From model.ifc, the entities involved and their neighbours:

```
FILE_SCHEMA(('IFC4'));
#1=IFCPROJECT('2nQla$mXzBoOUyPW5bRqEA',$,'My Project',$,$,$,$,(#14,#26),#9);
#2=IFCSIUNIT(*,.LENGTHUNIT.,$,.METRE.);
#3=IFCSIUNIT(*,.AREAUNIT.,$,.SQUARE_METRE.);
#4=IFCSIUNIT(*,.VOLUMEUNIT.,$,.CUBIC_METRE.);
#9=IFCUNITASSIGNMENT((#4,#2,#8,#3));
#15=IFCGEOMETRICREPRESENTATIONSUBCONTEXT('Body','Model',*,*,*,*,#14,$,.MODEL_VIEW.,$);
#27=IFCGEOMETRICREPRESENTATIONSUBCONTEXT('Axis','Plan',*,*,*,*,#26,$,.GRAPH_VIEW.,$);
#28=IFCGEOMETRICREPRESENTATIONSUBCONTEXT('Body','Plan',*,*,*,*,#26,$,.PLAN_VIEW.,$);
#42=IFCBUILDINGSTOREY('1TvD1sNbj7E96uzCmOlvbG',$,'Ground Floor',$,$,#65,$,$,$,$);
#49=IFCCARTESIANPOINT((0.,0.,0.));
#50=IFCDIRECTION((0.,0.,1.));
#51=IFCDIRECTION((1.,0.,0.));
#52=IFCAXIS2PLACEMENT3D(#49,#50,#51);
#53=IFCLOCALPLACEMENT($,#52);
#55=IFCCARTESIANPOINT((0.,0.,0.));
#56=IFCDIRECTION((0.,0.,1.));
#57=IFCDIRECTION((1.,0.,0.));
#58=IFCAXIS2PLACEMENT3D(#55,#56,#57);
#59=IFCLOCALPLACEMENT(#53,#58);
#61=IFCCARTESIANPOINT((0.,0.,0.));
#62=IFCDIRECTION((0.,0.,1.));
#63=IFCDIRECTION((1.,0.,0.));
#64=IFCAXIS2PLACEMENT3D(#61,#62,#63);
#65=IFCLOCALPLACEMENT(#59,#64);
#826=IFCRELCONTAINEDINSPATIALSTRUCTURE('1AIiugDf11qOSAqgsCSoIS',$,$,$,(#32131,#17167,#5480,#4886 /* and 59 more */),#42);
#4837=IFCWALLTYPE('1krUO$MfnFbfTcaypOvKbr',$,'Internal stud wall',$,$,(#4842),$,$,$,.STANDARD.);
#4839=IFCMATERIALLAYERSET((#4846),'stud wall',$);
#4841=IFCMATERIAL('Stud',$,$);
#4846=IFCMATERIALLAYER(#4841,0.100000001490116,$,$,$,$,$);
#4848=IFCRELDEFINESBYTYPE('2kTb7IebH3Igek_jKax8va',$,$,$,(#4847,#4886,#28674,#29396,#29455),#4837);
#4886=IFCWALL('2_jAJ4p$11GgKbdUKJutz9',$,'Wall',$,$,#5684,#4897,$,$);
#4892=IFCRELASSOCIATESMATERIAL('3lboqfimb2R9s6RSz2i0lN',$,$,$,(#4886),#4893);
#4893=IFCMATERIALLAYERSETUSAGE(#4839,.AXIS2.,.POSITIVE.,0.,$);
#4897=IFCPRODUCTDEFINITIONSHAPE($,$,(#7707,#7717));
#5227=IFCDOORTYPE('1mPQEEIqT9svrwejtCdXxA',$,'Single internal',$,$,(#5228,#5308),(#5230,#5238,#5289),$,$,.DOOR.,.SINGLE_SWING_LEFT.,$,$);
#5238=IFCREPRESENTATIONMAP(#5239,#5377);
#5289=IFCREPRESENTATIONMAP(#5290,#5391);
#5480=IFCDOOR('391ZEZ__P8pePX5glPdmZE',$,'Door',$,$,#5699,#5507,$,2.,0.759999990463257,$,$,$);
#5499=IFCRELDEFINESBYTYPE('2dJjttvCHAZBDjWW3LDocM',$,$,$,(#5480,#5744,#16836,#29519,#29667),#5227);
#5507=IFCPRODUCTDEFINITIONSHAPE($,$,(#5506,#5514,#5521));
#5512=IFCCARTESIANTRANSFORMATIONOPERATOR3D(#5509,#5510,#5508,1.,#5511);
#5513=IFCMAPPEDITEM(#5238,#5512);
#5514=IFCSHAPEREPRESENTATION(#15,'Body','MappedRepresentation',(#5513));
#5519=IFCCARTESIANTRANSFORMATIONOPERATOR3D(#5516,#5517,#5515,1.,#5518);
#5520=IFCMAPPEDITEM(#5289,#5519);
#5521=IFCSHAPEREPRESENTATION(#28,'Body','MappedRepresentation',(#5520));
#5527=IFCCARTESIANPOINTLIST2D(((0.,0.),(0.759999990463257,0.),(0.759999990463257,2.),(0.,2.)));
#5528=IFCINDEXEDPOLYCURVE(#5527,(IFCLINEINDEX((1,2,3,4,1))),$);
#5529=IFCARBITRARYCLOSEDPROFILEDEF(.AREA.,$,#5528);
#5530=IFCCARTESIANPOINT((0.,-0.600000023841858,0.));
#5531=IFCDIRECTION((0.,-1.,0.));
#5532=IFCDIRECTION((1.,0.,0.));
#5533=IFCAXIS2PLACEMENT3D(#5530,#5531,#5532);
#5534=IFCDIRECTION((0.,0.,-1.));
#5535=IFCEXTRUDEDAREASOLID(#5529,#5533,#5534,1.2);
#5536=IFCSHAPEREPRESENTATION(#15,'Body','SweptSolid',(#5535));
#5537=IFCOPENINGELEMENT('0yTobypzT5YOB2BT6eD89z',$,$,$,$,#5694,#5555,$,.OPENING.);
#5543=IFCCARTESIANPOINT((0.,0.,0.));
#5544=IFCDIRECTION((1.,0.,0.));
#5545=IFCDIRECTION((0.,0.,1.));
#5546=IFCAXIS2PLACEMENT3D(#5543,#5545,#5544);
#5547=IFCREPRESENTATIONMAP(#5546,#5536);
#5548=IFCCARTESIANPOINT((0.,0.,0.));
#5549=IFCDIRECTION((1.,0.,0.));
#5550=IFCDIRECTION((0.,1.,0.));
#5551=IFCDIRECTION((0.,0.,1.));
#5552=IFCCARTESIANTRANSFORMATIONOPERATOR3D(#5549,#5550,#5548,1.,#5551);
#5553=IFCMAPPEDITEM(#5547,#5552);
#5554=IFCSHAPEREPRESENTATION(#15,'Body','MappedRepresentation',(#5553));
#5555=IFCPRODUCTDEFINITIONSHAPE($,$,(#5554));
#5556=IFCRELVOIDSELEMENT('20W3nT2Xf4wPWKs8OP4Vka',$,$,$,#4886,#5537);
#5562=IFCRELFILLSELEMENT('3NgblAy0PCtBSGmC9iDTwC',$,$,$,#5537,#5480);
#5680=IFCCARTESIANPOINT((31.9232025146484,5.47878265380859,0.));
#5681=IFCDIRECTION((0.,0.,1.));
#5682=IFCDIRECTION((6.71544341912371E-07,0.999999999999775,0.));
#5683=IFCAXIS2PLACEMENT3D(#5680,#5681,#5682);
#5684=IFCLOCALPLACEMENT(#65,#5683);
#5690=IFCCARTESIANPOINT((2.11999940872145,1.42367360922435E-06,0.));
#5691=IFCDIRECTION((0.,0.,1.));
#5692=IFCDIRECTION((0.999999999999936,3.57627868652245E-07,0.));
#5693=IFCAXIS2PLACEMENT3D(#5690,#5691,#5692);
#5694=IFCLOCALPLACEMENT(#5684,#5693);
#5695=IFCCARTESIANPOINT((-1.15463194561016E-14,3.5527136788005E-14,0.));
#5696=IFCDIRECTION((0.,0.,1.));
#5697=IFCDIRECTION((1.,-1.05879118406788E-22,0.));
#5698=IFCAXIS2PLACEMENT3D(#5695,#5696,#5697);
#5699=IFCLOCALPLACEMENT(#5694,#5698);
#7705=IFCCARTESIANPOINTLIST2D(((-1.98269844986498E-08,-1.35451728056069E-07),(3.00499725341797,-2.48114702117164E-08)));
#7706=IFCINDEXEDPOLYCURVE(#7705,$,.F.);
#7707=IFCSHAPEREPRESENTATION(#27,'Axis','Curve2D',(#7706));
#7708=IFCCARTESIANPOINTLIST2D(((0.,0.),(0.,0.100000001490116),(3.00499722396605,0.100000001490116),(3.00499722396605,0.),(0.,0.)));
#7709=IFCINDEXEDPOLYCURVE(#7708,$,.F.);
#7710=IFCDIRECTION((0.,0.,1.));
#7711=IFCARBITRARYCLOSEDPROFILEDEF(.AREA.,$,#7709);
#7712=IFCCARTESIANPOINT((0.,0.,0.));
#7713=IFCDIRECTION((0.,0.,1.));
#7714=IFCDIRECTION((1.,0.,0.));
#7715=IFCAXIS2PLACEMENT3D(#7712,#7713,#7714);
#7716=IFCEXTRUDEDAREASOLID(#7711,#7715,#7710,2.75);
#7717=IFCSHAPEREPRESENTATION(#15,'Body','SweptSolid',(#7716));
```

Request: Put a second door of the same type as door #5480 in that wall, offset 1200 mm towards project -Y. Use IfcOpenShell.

```python
import ifcopenshell
import ifcopenshell.api.feature
import ifcopenshell.api.geometry
import ifcopenshell.api.root
import ifcopenshell.geom
import ifcopenshell.util.element
import ifcopenshell.util.placement
import ifcopenshell.util.shape
import ifcopenshell.util.unit

model = ifcopenshell.open("model.ifc")
unit_scale = ifcopenshell.util.unit.calculate_unit_scale(model)
settings = ifcopenshell.geom.settings()


def volume(element):
    """Net volume in cubic metres, openings subtracted."""
    shape = ifcopenshell.geom.create_shape(settings, element)
    return ifcopenshell.util.shape.get_volume(shape.geometry)


door = model.by_guid("391ZEZ__P8pePX5glPdmZE")
opening = door.FillsVoids[0].RelatingOpeningElement
wall = opening.VoidsElements[0].RelatingBuildingElement
before = volume(wall)
shift = ifcopenshell.util.placement.get_local_placement(wall.ObjectPlacement)[:3, 0] * -1.2 / unit_scale

# copy_class copies the void relationship, type, container and properties, but no geometry.
new_opening = ifcopenshell.api.root.copy_class(model, product=opening)
new_opening.Representation = ifcopenshell.util.element.copy_deep(
    model, opening.Representation, exclude=["IfcGeometricRepresentationContext", "IfcRepresentationMap"]
)
new_door = ifcopenshell.api.root.copy_class(model, product=door)
new_door.Representation = ifcopenshell.util.element.copy_deep(
    model, door.Representation, exclude=["IfcGeometricRepresentationContext", "IfcRepresentationMap"]
)
ifcopenshell.api.feature.add_filling(model, opening=new_opening, element=new_door)

for old, new in ((opening, new_opening), (door, new_door)):
    matrix = ifcopenshell.util.placement.get_local_placement(old.ObjectPlacement)
    matrix[:3, 3] += shift
    ifcopenshell.api.geometry.edit_object_placement(model, product=new, matrix=matrix, is_si=False)

after = volume(wall)

print(f"wall volume {before:.3f} -> {after:.3f} m3")

model.write("model_updated.ifc")
```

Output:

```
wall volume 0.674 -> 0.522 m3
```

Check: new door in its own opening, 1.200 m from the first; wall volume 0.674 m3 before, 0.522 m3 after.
